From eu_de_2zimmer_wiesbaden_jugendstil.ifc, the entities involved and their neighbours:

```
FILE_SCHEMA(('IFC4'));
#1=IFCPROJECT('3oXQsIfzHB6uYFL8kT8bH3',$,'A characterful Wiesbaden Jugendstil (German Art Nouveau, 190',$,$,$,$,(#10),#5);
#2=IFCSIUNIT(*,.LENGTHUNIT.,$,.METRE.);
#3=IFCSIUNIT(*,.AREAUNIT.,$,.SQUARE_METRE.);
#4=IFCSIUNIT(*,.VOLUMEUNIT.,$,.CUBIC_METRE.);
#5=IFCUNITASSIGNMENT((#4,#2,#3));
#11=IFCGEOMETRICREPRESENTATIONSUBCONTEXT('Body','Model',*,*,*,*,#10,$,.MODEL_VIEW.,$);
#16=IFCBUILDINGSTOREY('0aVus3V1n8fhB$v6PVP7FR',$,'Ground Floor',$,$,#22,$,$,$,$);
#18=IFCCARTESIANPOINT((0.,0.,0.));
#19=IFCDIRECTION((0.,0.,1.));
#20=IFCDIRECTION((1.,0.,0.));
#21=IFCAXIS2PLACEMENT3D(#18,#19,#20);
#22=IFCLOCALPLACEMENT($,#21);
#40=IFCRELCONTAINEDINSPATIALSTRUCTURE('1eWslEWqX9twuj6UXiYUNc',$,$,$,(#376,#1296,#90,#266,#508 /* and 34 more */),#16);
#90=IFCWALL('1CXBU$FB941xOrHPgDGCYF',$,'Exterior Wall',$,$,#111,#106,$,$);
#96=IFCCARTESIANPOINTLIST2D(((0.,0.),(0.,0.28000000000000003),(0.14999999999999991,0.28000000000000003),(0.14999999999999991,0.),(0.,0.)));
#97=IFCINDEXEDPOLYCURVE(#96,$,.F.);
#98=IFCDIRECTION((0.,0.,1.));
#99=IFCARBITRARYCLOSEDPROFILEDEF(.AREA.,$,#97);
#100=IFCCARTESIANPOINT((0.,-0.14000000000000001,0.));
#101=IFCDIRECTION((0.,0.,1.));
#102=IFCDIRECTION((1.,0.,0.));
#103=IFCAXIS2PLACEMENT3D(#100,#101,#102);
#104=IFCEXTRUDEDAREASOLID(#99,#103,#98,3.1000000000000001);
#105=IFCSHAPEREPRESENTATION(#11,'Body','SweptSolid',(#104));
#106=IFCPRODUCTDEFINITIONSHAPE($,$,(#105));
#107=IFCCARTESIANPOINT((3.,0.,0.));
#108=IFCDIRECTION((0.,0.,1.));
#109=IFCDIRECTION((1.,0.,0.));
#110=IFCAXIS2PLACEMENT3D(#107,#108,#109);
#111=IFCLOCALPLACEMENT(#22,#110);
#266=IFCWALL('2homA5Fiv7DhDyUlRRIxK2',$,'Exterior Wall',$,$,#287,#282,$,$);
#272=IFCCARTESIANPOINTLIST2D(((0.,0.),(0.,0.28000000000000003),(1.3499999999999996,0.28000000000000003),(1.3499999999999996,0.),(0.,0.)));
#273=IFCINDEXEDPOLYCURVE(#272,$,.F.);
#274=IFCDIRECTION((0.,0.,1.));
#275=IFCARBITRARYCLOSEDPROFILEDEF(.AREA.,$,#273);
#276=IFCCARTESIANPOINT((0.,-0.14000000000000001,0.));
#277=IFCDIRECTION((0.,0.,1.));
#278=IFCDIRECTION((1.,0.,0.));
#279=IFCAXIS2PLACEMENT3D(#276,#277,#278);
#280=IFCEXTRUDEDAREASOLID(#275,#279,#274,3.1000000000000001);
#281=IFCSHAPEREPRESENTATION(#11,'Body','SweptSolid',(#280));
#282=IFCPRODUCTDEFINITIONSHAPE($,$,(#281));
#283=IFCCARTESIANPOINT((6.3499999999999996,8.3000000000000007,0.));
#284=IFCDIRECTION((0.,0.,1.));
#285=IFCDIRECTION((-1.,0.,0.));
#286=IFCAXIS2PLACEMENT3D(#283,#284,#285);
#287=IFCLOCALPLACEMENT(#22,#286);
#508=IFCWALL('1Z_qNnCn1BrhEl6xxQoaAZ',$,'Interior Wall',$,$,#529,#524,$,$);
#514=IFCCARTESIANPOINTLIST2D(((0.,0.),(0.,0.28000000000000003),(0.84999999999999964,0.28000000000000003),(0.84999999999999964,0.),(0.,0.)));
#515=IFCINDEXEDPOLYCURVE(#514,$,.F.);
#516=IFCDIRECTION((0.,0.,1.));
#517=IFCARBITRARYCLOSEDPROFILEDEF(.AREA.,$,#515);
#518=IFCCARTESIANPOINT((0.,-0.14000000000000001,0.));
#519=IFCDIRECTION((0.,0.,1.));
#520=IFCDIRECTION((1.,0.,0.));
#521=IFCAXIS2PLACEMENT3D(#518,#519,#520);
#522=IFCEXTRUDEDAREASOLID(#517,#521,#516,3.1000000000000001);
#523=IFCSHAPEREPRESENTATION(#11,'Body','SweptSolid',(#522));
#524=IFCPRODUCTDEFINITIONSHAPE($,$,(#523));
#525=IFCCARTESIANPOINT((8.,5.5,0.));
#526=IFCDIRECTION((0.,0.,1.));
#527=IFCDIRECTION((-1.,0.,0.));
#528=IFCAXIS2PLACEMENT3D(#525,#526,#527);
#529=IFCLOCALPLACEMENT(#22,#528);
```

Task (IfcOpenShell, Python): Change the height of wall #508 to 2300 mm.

```python
import ifcopenshell
import ifcopenshell.geom
import ifcopenshell.util.representation
import ifcopenshell.util.shape
import ifcopenshell.util.unit

model = ifcopenshell.open("eu_de_2zimmer_wiesbaden_jugendstil.ifc")
unit_scale = ifcopenshell.util.unit.calculate_unit_scale(model)
settings = ifcopenshell.geom.settings()


def volume(element):
    """Net volume in cubic metres, openings subtracted."""
    shape = ifcopenshell.geom.create_shape(settings, element)
    return ifcopenshell.util.shape.get_volume(shape.geometry)


wall = model.by_guid("1Z_qNnCn1BrhEl6xxQoaAZ")
before = volume(wall)

body = ifcopenshell.util.representation.get_representation(wall, "Model", "Body")
solid = body.Items[0]
old_height = solid.Depth
solid.Depth = 2.3 / unit_scale
after = volume(wall)

print(f"height {old_height:g} -> {solid.Depth:g}, volume {before:.3f} -> {after:.3f} m3")

model.write("eu_de_2zimmer_wiesbaden_jugendstil_v2.ifc")
```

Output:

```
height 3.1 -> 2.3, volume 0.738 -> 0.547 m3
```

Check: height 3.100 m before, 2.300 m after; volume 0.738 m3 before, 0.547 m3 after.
